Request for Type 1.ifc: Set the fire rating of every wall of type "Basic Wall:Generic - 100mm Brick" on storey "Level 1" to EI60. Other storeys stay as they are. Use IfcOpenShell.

First a look at what the model holds.

```python
import ifcopenshell
import ifcopenshell.util.element

model = ifcopenshell.open("Type 1.ifc")
print(model.schema)
storey = next(s for s in model.by_type("IfcBuildingStorey") if s.Name == "Level 1")
walls = [e for e in ifcopenshell.util.element.get_decomposition(storey) if e.is_a("IfcWall")]
seen = {}
for e in walls:
    element_type = ifcopenshell.util.element.get_type(e)
    key = (element_type.Name if element_type != e and element_type else None, ifcopenshell.util.element.get_pset(e, "Pset_WallCommon", "FireRating"))
    seen[key] = seen.get(key, 0) + 1
for (name, value), count in sorted(seen.items(), key=str):
    print(count, "x", name, "|", value)
```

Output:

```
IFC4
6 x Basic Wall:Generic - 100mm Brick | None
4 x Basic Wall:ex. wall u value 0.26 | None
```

```python
import ifcopenshell
import ifcopenshell.api.pset
import ifcopenshell.util.element

model = ifcopenshell.open("Type 1.ifc")

storey = next(s for s in model.by_type("IfcBuildingStorey") if s.Name == "Level 1")
walls = [e for e in ifcopenshell.util.element.get_decomposition(storey) if e.is_a("IfcWall")]

count = 0
for e in walls:
    element_type = ifcopenshell.util.element.get_type(e)
    if element_type in (None, e) or element_type.Name != "Basic Wall:Generic - 100mm Brick":
        continue
    # add_pset returns the element's existing set when there is one.
    pset = ifcopenshell.api.pset.add_pset(model, product=e, name="Pset_WallCommon")
    ifcopenshell.api.pset.edit_pset(model, pset=pset, properties={"FireRating": "EI60"})
    count += 1

print(count, "walls updated")

model.write("Type 1_edited.ifc")
```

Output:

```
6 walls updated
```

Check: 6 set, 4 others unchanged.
